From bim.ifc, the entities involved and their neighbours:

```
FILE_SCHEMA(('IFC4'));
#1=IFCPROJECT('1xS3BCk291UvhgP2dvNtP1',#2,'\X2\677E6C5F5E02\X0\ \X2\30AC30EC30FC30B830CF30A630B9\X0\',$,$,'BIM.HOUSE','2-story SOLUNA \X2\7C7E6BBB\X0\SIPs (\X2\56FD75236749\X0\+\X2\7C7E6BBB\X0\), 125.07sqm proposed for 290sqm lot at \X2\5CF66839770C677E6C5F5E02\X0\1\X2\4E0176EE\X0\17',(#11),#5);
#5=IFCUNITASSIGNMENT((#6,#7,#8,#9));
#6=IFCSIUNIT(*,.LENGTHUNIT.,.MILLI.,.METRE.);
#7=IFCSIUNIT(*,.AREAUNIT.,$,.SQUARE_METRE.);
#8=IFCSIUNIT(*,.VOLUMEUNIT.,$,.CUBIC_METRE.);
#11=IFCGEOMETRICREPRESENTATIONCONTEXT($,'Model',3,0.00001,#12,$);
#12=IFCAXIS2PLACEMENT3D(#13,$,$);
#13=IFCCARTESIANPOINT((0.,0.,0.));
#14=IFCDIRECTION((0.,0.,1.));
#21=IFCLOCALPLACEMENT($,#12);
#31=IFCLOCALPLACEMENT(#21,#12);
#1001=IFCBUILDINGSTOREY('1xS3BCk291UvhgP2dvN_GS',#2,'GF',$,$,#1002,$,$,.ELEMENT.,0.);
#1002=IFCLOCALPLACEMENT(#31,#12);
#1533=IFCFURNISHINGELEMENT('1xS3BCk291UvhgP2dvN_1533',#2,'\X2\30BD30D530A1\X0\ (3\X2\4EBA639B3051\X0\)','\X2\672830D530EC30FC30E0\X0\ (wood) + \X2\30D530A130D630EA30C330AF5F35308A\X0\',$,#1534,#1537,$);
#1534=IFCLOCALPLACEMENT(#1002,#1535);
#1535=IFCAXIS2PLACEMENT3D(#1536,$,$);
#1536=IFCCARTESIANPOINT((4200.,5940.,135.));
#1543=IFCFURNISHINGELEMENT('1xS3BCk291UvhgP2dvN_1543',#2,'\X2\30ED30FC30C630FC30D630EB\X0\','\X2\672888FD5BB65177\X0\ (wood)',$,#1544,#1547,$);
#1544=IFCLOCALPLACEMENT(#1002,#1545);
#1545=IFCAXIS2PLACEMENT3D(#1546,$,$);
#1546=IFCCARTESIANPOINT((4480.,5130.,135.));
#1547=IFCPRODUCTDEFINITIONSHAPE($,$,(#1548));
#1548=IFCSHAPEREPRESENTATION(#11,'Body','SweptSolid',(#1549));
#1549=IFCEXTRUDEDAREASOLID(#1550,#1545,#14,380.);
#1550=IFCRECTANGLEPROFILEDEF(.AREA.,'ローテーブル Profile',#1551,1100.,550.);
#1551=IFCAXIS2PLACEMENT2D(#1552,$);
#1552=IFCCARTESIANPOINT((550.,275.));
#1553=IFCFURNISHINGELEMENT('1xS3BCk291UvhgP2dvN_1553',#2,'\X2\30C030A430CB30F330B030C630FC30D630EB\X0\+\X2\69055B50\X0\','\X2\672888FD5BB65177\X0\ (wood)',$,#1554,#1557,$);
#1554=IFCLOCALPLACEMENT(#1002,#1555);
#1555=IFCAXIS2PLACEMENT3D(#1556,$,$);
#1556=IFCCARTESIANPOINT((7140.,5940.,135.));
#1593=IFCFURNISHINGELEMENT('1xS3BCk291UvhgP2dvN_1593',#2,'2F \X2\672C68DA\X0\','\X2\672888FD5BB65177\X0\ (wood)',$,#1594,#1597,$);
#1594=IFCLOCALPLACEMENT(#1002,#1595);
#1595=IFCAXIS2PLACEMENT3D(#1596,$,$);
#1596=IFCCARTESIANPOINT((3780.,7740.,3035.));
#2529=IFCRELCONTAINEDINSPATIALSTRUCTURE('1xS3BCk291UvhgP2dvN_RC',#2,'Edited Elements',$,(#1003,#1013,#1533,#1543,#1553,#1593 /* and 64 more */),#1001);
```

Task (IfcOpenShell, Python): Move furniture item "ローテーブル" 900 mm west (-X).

```python
import ifcopenshell
import ifcopenshell.api.geometry
import ifcopenshell.util.placement
import ifcopenshell.util.unit

model = ifcopenshell.open("bim.ifc")
unit_scale = ifcopenshell.util.unit.calculate_unit_scale(model)

item = model.by_guid("1xS3BCk291UvhgP2dvN_1543")
matrix = ifcopenshell.util.placement.get_local_placement(item.ObjectPlacement)
matrix[0, 3] -= 0.9 / unit_scale
ifcopenshell.api.geometry.edit_object_placement(model, product=item, matrix=matrix, is_si=False)

print(ifcopenshell.util.placement.get_local_placement(item.ObjectPlacement).round(3) + 0.0)

model.write("bim_v2.ifc")
```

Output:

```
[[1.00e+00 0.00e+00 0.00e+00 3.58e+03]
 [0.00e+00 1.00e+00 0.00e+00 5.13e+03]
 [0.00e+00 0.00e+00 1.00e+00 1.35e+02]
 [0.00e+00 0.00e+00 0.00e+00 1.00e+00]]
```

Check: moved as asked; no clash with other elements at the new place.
